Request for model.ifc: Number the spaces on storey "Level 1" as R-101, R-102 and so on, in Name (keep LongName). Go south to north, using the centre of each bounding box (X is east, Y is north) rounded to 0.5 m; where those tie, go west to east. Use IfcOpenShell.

First a look at what the model holds.

```python
import ifcopenshell
import ifcopenshell.util.element
import ifcopenshell.util.placement

model = ifcopenshell.open("model.ifc")
print(model.schema)
storey = next(s for s in model.by_type("IfcBuildingStorey") if s.Name == "Level 1")
spaces = [e for e in ifcopenshell.util.element.get_decomposition(storey) if e.is_a("IfcSpace")]
for e in sorted(spaces, key=lambda e: e.id()):
    origin = ifcopenshell.util.placement.get_local_placement(e.ObjectPlacement)[:3, 3]
    print(e.id(), e.Name, e.LongName, origin.round(2) + 0.0, sep=" | ")
```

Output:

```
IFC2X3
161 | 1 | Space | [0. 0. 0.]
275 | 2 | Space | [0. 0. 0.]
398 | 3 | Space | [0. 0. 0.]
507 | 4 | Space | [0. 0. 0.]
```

```python
import ifcopenshell
import ifcopenshell.geom
import ifcopenshell.util.element
import ifcopenshell.util.shape

model = ifcopenshell.open("model.ifc")
settings = ifcopenshell.geom.settings()
settings.set("use-world-coords", True)


def centre(element):
    shape = ifcopenshell.geom.create_shape(settings, element)
    return ifcopenshell.util.shape.get_bbox_centroid(shape.geometry)


storey = next(s for s in model.by_type("IfcBuildingStorey") if s.Name == "Level 1")
spaces = [e for e in ifcopenshell.util.element.get_decomposition(storey) if e.is_a("IfcSpace")]

# Insertion points can sit at a corner or the storey origin, so sort by the geometry (in metres).
centres = {e: centre(e) for e in spaces}
spaces.sort(key=lambda e: (round(centres[e][1] / 0.5), centres[e][0]))

for i, e in enumerate(spaces, start=1):
    number = f"R-1{i:02d}"
    e.Name = number
    print(e.id(), number)

model.write("model_edited.ifc")
```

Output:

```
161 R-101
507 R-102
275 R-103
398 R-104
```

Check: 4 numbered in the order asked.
